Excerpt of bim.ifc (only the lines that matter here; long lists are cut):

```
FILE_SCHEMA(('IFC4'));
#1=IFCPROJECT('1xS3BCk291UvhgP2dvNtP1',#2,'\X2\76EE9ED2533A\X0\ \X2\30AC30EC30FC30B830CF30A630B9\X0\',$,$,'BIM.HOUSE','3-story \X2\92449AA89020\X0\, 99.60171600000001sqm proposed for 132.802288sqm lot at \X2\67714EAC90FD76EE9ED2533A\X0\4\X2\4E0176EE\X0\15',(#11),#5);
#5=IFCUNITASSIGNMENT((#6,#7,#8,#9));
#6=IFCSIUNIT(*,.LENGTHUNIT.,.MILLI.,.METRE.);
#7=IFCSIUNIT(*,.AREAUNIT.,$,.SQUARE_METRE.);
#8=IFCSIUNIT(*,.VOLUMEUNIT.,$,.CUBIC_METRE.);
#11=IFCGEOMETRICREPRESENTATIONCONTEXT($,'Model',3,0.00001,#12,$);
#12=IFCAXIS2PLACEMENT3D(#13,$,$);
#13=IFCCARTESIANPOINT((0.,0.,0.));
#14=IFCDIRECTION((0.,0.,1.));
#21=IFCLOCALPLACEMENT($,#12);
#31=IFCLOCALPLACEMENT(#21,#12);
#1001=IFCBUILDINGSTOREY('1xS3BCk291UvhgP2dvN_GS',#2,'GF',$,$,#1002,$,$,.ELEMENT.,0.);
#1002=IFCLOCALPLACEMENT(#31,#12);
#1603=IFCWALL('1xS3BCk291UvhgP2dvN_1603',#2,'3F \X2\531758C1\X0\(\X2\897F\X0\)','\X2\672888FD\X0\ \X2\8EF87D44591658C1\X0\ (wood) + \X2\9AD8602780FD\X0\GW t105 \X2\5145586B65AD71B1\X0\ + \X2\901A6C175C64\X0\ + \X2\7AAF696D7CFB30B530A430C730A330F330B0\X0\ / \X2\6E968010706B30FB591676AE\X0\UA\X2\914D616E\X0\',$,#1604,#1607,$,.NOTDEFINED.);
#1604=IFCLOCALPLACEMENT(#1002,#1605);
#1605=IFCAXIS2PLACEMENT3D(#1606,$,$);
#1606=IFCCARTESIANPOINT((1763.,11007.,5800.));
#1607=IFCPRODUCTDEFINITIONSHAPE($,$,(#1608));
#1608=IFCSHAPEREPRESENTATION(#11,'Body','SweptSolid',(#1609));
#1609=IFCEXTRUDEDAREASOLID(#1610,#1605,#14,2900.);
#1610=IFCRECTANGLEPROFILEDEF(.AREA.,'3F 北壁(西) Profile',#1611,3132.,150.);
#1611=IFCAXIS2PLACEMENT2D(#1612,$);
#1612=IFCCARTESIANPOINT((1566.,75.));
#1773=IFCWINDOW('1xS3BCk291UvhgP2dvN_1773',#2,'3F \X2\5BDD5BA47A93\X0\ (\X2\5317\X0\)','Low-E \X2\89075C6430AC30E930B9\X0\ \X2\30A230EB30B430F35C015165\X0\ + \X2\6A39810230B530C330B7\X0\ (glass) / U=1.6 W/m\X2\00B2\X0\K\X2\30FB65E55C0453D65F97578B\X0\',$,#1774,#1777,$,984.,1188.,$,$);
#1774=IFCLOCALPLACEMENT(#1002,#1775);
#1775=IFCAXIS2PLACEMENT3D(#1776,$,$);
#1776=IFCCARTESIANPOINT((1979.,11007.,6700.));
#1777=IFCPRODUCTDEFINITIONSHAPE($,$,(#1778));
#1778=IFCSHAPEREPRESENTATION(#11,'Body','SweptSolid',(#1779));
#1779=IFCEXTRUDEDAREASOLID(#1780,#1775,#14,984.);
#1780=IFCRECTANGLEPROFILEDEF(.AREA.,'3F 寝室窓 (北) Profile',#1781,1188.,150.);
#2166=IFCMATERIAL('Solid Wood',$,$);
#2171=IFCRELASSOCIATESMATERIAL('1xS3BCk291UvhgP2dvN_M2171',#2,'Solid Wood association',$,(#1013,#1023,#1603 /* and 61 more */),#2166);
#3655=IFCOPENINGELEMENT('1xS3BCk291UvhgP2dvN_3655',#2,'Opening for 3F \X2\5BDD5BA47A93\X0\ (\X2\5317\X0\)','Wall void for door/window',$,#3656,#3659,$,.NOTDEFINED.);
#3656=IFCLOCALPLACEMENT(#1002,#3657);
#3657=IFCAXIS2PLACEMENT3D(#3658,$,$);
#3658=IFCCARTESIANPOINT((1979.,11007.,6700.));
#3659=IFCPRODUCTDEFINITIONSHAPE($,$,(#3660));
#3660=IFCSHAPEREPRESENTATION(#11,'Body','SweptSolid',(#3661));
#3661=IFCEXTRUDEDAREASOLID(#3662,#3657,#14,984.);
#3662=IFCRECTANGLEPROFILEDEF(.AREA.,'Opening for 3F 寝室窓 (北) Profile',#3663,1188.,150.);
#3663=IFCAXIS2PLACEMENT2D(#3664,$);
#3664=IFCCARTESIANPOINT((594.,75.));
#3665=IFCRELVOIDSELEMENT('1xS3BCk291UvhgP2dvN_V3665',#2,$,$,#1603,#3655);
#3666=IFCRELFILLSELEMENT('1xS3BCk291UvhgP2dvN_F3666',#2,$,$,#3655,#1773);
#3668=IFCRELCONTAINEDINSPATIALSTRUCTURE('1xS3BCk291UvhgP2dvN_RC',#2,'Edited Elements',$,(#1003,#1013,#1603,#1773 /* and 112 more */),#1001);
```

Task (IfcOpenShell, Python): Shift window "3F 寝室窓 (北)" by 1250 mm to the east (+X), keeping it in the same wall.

```python
import ifcopenshell
import ifcopenshell.api.geometry
import ifcopenshell.util.placement
import ifcopenshell.util.unit

model = ifcopenshell.open("bim.ifc")
unit_scale = ifcopenshell.util.unit.calculate_unit_scale(model)

window = model.by_id(1773)
opening = window.FillsVoids[0].RelatingOpeningElement
wall = opening.VoidsElements[0].RelatingBuildingElement

wall_matrix = ifcopenshell.util.placement.get_local_placement(wall.ObjectPlacement)
shift = wall_matrix[:3, 0] * 1.25 / unit_scale
before = ifcopenshell.util.placement.get_local_placement(window.ObjectPlacement)[:3, 3].copy()

# The window is not placed relative to its opening, so move both.
for product in (opening, window):
    matrix = ifcopenshell.util.placement.get_local_placement(product.ObjectPlacement)
    matrix[:3, 3] += shift
    ifcopenshell.api.geometry.edit_object_placement(model, product=product, matrix=matrix, is_si=False)

after = ifcopenshell.util.placement.get_local_placement(window.ObjectPlacement)[:3, 3]
print("window moved by", (after - before).round(3) + 0.0)

model.write("bim-out.ifc")
```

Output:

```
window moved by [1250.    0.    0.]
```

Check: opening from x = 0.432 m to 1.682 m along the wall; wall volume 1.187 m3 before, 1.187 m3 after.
